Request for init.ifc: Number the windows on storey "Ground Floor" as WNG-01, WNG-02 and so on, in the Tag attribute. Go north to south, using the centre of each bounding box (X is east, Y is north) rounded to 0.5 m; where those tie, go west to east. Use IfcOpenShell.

First a look at what the model holds.

```python
import ifcopenshell
import ifcopenshell.util.element
import ifcopenshell.util.placement

model = ifcopenshell.open("init.ifc")
print(model.schema)
storey = next(s for s in model.by_type("IfcBuildingStorey") if s.Name == "Ground Floor")
windows = [e for e in ifcopenshell.util.element.get_decomposition(storey) if e.is_a("IfcWindow")]
for e in sorted(windows, key=lambda e: e.id()):
    origin = ifcopenshell.util.placement.get_local_placement(e.ObjectPlacement)[:3, 3]
    print(e.id(), e.Tag, e.Name, origin.round(2) + 0.0, sep=" | ")
```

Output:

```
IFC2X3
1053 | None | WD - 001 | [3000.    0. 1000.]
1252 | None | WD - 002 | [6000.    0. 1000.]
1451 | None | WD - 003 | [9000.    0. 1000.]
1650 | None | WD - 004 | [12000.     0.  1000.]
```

```python
import ifcopenshell
import ifcopenshell.geom
import ifcopenshell.util.element
import ifcopenshell.util.shape

model = ifcopenshell.open("init.ifc")
settings = ifcopenshell.geom.settings()
settings.set("use-world-coords", True)


def centre(element):
    shape = ifcopenshell.geom.create_shape(settings, element)
    return ifcopenshell.util.shape.get_bbox_centroid(shape.geometry)


storey = next(s for s in model.by_type("IfcBuildingStorey") if s.Name == "Ground Floor")
windows = [e for e in ifcopenshell.util.element.get_decomposition(storey) if e.is_a("IfcWindow")]

# Insertion points can sit at a corner or the storey origin, so sort by the geometry (in metres).
centres = {e: centre(e) for e in windows}
windows.sort(key=lambda e: (-round(centres[e][1] / 0.5), centres[e][0]))

for i, e in enumerate(windows, start=1):
    number = f"WNG-{i:02d}"
    e.Tag = number
    print(e.id(), number)

model.write("init_edited.ifc")
```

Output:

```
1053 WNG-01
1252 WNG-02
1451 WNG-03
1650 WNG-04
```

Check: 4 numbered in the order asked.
